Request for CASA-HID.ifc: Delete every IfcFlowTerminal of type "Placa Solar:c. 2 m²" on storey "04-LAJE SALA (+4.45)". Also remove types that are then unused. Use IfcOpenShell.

First a look at what the model holds.

```python
import ifcopenshell
import ifcopenshell.util.element

model = ifcopenshell.open("CASA-HID.ifc")
print(model.schema)
storey = next(s for s in model.by_type("IfcBuildingStorey") if s.Name == "04-LAJE SALA (+4.45)")
terminals = [e for e in ifcopenshell.util.element.get_decomposition(storey) if e.is_a("IfcFlowTerminal")]
seen = {}
for e in terminals:
    element_type = ifcopenshell.util.element.get_type(e)
    name = element_type.Name if element_type not in (None, e) else None
    seen[name] = seen.get(name, 0) + 1
for name, count in sorted(seen.items(), key=str):
    print(count, "x", name)
```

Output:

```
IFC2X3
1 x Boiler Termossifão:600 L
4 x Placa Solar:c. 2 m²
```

```python
import ifcopenshell
import ifcopenshell.api.root
import ifcopenshell.util.element

model = ifcopenshell.open("CASA-HID.ifc")

storey = next(s for s in model.by_type("IfcBuildingStorey") if s.Name == "04-LAJE SALA (+4.45)")
terminals = [e for e in ifcopenshell.util.element.get_decomposition(storey) if e.is_a("IfcFlowTerminal")]
targets = [e for e in terminals if (t := ifcopenshell.util.element.get_type(e)) not in (None, e) and t.Name == "Placa Solar:c. 2 m²"]
types = {ifcopenshell.util.element.get_type(e) for e in targets} - {None, *targets}

for e in targets:
    ifcopenshell.api.root.remove_product(model, product=e)
print(len(targets), "removed")

unused = [t for t in types if not ifcopenshell.util.element.get_types(t)]
for t in unused:
    ifcopenshell.api.root.remove_product(model, product=t)
print(len(unused), "unused types removed")

model.write("CASA-HID_updated.ifc")
```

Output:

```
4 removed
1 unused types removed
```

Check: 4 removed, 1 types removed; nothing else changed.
